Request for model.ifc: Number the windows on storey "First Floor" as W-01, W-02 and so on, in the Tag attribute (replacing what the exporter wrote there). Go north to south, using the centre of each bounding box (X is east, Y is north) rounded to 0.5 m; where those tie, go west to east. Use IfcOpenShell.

First a look at what the model holds.

```python
import ifcopenshell
import ifcopenshell.util.element
import ifcopenshell.util.placement

model = ifcopenshell.open("model.ifc")
print(model.schema)
storey = next(s for s in model.by_type("IfcBuildingStorey") if s.Name == "First Floor")
windows = [e for e in ifcopenshell.util.element.get_decomposition(storey) if e.is_a("IfcWindow")]
for e in sorted(windows, key=lambda e: e.id()):
    origin = ifcopenshell.util.placement.get_local_placement(e.ObjectPlacement)[:3, 3]
    print(e.id(), e.Tag, e.Name, origin.round(2) + 0.0, sep=" | ")
```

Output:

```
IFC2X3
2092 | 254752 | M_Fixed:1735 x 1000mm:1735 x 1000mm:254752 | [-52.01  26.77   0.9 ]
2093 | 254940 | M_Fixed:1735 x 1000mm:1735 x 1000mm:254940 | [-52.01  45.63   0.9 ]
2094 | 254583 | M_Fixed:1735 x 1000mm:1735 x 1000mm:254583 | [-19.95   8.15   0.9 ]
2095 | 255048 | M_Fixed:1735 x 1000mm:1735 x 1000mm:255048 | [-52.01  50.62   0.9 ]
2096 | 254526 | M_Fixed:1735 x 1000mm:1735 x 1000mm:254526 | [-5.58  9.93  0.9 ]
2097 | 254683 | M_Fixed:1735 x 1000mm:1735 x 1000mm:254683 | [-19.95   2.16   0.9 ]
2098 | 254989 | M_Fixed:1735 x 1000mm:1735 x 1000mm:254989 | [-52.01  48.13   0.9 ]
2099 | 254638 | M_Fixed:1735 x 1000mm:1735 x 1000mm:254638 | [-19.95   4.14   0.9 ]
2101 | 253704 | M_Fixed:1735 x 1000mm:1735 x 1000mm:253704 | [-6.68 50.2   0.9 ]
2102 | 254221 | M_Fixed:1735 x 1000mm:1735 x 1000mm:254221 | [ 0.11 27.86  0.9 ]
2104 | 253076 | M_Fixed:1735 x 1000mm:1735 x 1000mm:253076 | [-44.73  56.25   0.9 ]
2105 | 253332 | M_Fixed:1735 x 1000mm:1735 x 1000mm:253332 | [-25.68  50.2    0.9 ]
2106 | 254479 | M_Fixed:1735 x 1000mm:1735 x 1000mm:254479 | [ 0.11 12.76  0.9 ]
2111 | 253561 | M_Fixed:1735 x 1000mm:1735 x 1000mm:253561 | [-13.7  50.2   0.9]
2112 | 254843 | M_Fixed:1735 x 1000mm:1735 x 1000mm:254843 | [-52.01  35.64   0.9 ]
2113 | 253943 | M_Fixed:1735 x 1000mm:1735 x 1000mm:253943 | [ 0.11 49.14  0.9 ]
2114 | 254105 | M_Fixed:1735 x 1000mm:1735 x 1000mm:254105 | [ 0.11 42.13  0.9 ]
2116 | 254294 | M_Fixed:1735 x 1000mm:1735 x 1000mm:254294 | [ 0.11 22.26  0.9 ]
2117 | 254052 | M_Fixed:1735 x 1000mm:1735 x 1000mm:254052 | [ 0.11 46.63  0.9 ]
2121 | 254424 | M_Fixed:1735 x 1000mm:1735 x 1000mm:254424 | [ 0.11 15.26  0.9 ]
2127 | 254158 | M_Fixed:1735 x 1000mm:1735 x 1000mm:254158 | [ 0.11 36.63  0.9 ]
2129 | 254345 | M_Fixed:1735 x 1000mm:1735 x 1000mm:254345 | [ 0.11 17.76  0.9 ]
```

```python
import ifcopenshell
import ifcopenshell.geom
import ifcopenshell.util.element
import ifcopenshell.util.shape

model = ifcopenshell.open("model.ifc")
settings = ifcopenshell.geom.settings()
settings.set("use-world-coords", True)


def centre(element):
    shape = ifcopenshell.geom.create_shape(settings, element)
    return ifcopenshell.util.shape.get_bbox_centroid(shape.geometry)


storey = next(s for s in model.by_type("IfcBuildingStorey") if s.Name == "First Floor")
windows = [e for e in ifcopenshell.util.element.get_decomposition(storey) if e.is_a("IfcWindow")]

# Insertion points can sit at a corner or the storey origin, so sort by the geometry (in metres).
centres = {e: centre(e) for e in windows}
windows.sort(key=lambda e: (-round(centres[e][1] / 0.5), centres[e][0]))

for i, e in enumerate(windows, start=1):
    number = f"W-{i:02d}"
    e.Tag = number
    print(e.id(), number)

model.write("model_edited.ifc")
```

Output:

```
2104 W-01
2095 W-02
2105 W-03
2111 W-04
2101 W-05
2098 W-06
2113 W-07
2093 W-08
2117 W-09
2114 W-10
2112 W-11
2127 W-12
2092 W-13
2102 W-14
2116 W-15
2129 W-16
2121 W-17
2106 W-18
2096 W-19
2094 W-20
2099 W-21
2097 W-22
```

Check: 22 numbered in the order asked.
